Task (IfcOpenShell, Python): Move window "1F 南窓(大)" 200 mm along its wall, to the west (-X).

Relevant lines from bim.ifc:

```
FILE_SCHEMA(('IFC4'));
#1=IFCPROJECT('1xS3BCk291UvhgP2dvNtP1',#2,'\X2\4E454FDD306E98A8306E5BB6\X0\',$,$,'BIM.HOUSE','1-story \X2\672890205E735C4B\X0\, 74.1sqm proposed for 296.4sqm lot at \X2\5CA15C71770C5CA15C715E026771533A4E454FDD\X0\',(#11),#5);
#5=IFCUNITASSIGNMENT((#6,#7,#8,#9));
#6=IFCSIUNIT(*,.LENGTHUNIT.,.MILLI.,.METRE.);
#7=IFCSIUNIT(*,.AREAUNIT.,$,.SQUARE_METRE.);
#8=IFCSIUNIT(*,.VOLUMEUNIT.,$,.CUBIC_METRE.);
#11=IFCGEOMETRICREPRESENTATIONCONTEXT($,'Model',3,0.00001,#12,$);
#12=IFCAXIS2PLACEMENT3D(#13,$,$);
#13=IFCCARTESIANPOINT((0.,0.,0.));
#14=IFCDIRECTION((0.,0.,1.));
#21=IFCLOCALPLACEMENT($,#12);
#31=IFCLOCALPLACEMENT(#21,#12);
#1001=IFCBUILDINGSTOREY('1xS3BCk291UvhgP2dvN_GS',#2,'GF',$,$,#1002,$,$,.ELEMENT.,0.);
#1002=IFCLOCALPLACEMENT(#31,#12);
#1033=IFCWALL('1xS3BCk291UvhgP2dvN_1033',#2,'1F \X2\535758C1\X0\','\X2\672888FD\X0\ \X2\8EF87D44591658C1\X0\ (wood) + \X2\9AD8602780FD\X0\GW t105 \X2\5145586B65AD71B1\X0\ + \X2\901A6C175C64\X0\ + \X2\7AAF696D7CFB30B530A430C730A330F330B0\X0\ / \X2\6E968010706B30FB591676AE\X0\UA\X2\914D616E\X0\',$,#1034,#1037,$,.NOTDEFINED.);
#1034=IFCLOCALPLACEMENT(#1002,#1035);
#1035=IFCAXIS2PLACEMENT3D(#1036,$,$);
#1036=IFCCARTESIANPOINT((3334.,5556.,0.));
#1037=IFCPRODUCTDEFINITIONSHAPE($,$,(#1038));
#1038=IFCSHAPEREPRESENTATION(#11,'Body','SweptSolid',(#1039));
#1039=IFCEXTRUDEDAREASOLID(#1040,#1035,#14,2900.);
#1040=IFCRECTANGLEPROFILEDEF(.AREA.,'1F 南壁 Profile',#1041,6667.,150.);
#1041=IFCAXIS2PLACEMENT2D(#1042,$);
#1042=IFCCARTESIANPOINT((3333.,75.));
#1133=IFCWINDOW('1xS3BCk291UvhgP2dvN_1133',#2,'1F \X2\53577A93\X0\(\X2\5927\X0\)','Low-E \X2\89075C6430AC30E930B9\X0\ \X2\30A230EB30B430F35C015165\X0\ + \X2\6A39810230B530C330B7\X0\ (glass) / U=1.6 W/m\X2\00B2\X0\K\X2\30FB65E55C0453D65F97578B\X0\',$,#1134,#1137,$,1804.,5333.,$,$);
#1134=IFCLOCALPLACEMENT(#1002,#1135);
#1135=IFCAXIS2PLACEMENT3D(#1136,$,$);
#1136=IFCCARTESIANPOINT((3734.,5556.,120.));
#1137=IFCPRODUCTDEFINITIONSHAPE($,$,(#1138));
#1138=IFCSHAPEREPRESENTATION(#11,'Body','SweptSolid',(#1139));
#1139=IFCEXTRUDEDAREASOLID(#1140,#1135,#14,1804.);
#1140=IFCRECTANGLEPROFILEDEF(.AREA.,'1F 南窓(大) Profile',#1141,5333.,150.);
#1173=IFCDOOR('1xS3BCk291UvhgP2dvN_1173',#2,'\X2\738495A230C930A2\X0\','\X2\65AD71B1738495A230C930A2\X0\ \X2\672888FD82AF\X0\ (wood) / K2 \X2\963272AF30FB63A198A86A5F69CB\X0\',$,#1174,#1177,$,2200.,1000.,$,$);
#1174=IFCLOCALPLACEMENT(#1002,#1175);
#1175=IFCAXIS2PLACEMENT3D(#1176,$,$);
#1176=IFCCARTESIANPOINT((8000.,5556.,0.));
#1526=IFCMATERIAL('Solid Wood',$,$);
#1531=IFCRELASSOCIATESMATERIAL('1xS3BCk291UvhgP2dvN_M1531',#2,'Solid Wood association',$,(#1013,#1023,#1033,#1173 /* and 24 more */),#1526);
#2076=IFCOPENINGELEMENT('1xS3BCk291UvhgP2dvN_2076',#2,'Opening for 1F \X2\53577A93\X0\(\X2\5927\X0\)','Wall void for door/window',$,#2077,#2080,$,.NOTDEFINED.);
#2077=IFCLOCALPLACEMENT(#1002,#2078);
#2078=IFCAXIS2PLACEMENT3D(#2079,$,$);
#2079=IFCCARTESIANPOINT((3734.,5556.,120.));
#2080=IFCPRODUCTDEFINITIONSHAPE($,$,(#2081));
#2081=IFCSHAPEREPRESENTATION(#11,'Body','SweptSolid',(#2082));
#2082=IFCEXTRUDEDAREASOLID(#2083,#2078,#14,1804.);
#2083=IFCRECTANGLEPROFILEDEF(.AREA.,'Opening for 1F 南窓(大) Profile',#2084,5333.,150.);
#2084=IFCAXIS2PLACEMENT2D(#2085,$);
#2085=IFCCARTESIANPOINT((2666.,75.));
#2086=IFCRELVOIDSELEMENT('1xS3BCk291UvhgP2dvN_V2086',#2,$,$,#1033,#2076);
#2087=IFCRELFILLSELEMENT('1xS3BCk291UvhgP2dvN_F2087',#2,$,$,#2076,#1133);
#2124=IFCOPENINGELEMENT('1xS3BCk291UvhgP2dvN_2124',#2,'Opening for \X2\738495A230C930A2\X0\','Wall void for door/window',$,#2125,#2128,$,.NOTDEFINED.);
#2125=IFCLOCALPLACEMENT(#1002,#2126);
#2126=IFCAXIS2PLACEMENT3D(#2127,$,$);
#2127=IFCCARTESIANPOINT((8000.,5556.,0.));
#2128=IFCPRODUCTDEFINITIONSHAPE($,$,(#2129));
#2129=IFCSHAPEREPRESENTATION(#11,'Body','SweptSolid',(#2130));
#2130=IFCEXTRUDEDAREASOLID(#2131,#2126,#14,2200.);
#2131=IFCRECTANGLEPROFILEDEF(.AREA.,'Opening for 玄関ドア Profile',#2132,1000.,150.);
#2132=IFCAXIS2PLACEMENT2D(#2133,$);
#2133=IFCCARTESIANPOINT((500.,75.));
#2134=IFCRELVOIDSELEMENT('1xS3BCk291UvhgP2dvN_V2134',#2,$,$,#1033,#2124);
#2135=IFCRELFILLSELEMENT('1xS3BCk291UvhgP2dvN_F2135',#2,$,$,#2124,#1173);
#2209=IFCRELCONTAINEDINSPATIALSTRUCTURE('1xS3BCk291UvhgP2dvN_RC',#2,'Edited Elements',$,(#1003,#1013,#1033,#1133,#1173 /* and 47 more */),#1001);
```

```python
import ifcopenshell
import ifcopenshell.api.geometry
import ifcopenshell.util.placement
import ifcopenshell.util.unit

model = ifcopenshell.open("bim.ifc")
unit_scale = ifcopenshell.util.unit.calculate_unit_scale(model)

window = model.by_id(1133)
opening = window.FillsVoids[0].RelatingOpeningElement
wall = opening.VoidsElements[0].RelatingBuildingElement

wall_matrix = ifcopenshell.util.placement.get_local_placement(wall.ObjectPlacement)
shift = wall_matrix[:3, 0] * -0.2 / unit_scale
before = ifcopenshell.util.placement.get_local_placement(window.ObjectPlacement)[:3, 3].copy()

# The window is not placed relative to its opening, so move both.
for product in (opening, window):
    matrix = ifcopenshell.util.placement.get_local_placement(product.ObjectPlacement)
    matrix[:3, 3] += shift
    ifcopenshell.api.geometry.edit_object_placement(model, product=product, matrix=matrix, is_si=False)

after = ifcopenshell.util.placement.get_local_placement(window.ObjectPlacement)[:3, 3]
print("window moved by", (after - before).round(3) + 0.0)

model.write("bim_edited.ifc")
```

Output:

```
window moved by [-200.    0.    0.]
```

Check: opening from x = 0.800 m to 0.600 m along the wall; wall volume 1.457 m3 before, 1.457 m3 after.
